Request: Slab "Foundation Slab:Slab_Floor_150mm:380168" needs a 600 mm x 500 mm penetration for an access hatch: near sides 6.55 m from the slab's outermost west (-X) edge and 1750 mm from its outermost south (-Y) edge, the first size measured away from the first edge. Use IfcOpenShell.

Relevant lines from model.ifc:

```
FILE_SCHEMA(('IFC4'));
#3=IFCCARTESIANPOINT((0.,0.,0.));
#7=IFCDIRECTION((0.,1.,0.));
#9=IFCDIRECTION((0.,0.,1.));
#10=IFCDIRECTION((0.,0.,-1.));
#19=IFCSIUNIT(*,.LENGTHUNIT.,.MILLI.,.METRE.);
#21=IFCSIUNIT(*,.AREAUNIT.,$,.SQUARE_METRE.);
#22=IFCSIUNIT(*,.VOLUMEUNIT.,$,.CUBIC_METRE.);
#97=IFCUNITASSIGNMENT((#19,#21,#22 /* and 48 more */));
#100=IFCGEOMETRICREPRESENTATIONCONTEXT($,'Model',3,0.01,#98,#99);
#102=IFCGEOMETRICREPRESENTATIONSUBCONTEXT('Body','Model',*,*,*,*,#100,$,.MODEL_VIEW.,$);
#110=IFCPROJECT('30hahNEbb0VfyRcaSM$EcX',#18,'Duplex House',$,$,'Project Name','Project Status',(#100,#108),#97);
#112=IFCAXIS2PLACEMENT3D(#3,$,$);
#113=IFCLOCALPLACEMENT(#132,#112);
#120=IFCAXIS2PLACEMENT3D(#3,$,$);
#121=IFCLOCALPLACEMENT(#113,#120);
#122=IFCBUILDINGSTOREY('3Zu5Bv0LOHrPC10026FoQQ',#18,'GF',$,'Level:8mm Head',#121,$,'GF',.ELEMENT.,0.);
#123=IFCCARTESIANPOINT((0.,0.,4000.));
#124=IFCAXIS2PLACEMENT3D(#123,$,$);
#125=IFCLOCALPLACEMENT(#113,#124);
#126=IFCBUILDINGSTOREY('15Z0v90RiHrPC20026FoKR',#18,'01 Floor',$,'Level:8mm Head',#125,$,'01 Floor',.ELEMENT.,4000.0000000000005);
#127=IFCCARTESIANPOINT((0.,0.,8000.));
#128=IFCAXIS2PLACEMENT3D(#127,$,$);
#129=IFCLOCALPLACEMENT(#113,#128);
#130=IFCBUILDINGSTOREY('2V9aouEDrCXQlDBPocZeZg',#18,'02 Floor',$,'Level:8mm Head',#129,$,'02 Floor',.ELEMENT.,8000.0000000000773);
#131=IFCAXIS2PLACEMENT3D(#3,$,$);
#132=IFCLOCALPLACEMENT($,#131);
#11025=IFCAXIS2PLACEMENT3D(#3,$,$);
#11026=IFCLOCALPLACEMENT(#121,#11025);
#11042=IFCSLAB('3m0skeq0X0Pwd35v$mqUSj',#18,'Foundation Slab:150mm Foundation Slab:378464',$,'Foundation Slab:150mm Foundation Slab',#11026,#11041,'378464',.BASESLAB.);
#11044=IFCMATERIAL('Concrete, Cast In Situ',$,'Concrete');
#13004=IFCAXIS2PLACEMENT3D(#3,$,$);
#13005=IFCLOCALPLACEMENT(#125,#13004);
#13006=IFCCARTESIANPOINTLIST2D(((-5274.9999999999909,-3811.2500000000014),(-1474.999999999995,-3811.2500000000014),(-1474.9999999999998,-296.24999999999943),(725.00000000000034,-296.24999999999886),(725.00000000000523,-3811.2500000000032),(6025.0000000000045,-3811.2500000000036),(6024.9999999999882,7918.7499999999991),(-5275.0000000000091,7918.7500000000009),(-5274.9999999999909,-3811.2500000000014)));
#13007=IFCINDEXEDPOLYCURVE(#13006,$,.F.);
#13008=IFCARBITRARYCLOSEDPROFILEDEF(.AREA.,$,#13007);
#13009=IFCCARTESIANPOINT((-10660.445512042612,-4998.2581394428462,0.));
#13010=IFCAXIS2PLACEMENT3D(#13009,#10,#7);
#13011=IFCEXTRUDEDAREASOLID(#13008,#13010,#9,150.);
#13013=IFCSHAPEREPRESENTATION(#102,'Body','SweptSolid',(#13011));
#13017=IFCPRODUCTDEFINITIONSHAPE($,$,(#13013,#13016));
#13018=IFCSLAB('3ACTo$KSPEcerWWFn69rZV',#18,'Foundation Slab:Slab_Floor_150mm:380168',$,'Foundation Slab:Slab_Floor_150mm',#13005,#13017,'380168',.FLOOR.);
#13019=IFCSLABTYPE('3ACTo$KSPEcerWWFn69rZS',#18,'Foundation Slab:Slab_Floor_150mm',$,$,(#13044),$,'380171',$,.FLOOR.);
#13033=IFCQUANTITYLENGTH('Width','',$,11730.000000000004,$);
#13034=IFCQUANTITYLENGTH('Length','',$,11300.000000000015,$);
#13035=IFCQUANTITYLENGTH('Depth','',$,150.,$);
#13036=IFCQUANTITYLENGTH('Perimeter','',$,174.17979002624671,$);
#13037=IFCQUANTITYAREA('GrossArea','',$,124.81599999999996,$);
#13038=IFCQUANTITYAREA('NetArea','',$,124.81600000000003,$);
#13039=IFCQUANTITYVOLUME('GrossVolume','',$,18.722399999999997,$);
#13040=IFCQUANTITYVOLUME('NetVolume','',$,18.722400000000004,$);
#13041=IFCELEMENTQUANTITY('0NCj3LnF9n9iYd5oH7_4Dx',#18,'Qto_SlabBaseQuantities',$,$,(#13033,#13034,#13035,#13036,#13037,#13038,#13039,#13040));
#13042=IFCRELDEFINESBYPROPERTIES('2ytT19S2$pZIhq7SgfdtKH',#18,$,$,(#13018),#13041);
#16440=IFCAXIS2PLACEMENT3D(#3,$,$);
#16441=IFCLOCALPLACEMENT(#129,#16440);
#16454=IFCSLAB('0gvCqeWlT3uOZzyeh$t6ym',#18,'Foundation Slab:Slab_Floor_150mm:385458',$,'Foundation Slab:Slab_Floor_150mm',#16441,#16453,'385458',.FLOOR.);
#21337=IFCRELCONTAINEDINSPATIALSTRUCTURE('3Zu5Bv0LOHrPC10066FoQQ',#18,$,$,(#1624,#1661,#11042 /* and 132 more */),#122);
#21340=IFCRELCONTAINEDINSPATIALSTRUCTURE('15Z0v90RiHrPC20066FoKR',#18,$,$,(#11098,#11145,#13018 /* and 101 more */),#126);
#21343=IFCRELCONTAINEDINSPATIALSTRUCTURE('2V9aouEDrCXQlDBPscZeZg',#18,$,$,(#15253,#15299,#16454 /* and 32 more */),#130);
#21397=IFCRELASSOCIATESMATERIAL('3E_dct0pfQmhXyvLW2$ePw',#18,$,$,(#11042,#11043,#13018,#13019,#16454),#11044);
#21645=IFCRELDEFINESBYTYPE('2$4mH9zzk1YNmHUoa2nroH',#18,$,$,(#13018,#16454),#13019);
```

```python
import numpy as np
import ifcopenshell
import ifcopenshell.api.feature
import ifcopenshell.api.geometry
import ifcopenshell.api.pset
import ifcopenshell.api.root
import ifcopenshell.geom
import ifcopenshell.util.element
import ifcopenshell.util.placement
import ifcopenshell.util.representation
import ifcopenshell.util.shape
import ifcopenshell.util.unit

model = ifcopenshell.open("model.ifc")
unit_scale = ifcopenshell.util.unit.calculate_unit_scale(model)
area_scale = ifcopenshell.util.unit.calculate_unit_scale(model, "AREAUNIT")
volume_scale = ifcopenshell.util.unit.calculate_unit_scale(model, "VOLUMEUNIT")
settings = ifcopenshell.geom.settings()


def volume(element):
    """Net volume in cubic metres, openings subtracted."""
    shape = ifcopenshell.geom.create_shape(settings, element)
    return ifcopenshell.util.shape.get_volume(shape.geometry)


slab = model.by_id(13018)
before = volume(slab)

# Extent in the slab's own axes, in metres. The edges named are its -X and -Y sides.
slab_shape = ifcopenshell.geom.create_shape(settings, slab)
vertices = ifcopenshell.util.shape.get_vertices(slab_shape.geometry)
x_min, y_min, bottom = vertices.min(axis=0)
top = vertices[:, 2].max()

opening = ifcopenshell.api.root.create_entity(model, ifc_class="IfcOpeningElement", name="Access hatch opening", predefined_type="OPENING")
context = ifcopenshell.util.representation.get_context(model, "Model", "Body", "MODEL_VIEW")
width, depth = 0.6, 0.5
outline = [(0.0, 0.0), (width, 0.0), (width, depth), (0.0, depth), (0.0, 0.0)]
# Overshoot both faces by 50 mm so the cut is clean.
shape = ifcopenshell.api.geometry.add_slab_representation(
    model, context=context, depth=top - bottom + 0.1, polyline=outline
)
ifcopenshell.api.geometry.assign_representation(model, product=opening, representation=shape)

matrix = ifcopenshell.util.placement.get_local_placement(slab.ObjectPlacement)
matrix[:, 3] = matrix @ np.append(np.array([x_min + 6.55, y_min + 1.75, bottom - 0.05]) / unit_scale, 1.0)
ifcopenshell.api.geometry.edit_object_placement(model, product=opening, matrix=matrix, is_si=False)
ifcopenshell.api.feature.add_feature(model, feature=opening, element=slab)

after = volume(slab)

# Update the slab's stored quantities.
qto = model.by_id(ifcopenshell.util.element.get_pset(slab, "Qto_SlabBaseQuantities", should_inherit=False)["id"])
ifcopenshell.api.pset.edit_qto(model, qto=qto, properties={
    "NetArea": after / (top - bottom) / area_scale,
    "NetVolume": after / volume_scale,
})

print(f"slab volume {before:.3f} -> {after:.3f} m3")

model.write("model-out.ifc")
```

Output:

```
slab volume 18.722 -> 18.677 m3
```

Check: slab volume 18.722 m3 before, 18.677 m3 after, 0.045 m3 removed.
